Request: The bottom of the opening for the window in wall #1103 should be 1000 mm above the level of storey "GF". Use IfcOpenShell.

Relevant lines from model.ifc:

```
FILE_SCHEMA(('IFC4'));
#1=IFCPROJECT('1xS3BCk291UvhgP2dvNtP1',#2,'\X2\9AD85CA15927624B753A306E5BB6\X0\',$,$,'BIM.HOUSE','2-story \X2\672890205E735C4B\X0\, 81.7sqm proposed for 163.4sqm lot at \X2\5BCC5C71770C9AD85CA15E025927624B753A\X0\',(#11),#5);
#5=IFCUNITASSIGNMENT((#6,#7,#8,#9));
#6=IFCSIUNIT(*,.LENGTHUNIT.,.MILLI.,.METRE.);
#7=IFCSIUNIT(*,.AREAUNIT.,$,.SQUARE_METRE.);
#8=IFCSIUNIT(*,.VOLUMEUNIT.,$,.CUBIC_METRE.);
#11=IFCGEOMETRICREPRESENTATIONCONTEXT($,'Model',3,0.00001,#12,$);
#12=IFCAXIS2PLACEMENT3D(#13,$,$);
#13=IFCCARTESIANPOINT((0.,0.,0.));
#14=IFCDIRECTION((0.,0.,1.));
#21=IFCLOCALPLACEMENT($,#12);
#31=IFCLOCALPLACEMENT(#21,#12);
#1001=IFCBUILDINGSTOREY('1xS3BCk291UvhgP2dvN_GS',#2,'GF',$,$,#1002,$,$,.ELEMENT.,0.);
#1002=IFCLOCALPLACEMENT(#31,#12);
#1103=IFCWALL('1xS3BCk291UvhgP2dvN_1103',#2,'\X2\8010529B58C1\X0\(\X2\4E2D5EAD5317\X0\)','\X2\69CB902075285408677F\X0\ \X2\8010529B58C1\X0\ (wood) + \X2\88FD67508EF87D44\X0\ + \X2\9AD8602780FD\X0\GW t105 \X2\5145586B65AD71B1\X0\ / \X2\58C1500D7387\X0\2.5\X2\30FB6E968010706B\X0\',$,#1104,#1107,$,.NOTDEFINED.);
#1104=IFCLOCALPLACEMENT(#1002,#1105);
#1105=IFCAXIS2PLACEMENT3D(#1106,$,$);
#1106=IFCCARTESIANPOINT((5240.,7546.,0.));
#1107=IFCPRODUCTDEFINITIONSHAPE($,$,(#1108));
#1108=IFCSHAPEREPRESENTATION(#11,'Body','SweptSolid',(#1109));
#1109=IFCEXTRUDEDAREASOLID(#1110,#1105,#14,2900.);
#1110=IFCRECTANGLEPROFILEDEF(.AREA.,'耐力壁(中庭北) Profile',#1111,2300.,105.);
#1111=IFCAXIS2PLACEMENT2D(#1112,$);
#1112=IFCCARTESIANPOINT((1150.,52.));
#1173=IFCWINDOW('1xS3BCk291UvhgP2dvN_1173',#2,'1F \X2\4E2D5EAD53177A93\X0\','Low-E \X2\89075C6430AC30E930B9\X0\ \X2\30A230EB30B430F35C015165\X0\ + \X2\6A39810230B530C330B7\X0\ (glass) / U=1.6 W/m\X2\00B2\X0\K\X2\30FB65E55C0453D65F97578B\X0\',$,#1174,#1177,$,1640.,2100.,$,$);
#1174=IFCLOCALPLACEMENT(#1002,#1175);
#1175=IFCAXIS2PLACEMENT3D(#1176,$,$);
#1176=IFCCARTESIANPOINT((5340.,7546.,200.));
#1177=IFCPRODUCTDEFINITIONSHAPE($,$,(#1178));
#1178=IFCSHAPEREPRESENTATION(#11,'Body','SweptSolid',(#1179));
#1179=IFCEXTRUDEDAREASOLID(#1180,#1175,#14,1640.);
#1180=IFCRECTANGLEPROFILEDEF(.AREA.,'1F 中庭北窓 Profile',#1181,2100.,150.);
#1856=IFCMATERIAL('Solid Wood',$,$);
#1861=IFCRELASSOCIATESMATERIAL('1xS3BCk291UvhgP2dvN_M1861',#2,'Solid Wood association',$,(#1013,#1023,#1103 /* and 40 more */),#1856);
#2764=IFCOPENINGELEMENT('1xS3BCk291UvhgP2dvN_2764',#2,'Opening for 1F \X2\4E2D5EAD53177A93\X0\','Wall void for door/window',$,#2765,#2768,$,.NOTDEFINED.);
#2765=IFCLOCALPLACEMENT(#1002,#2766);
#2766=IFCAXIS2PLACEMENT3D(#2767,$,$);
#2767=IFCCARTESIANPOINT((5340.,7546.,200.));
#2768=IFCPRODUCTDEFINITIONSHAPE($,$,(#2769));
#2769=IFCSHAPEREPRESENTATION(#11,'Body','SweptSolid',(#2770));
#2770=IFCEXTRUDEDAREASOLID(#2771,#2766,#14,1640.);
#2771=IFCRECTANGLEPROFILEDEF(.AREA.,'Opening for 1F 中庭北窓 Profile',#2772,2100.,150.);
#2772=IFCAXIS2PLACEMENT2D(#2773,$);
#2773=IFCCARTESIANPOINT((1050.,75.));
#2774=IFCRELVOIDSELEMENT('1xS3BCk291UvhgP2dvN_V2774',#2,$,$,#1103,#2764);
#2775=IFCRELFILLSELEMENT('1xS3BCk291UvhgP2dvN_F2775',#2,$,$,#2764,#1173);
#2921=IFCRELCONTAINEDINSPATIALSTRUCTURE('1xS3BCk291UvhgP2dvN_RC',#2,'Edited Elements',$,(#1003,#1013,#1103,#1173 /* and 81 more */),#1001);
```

```python
import numpy as np
import ifcopenshell
import ifcopenshell.api.geometry
import ifcopenshell.geom
import ifcopenshell.util.element
import ifcopenshell.util.placement
import ifcopenshell.util.shape
import ifcopenshell.util.unit

model = ifcopenshell.open("model.ifc")
unit_scale = ifcopenshell.util.unit.calculate_unit_scale(model)

window = model.by_guid("1xS3BCk291UvhgP2dvN_1173")
opening = window.FillsVoids[0].RelatingOpeningElement
storey = ifcopenshell.util.element.get_container(window, ifc_class="IfcBuildingStorey")
level = ifcopenshell.util.placement.get_local_placement(storey.ObjectPlacement)[2, 3]

# The opening's origin need not be at the sill, so measure its lowest point.
shape = ifcopenshell.geom.create_shape(ifcopenshell.geom.settings(), opening)
bottom = ifcopenshell.util.shape.get_shape_bottom_elevation(shape, shape.geometry) / unit_scale
dz = level + 1 / unit_scale - bottom

shift = np.array([0.0, 0.0, dz])
# The window is not placed relative to its opening, so move both.
for product in (opening, window):
    matrix = ifcopenshell.util.placement.get_local_placement(product.ObjectPlacement)
    matrix[:3, 3] += shift
    ifcopenshell.api.geometry.edit_object_placement(model, product=product, matrix=matrix, is_si=False)

print(f"moved by {dz * unit_scale:+.3f} m")

model.write("model_edited.ifc")
```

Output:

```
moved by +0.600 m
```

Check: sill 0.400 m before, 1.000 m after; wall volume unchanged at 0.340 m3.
